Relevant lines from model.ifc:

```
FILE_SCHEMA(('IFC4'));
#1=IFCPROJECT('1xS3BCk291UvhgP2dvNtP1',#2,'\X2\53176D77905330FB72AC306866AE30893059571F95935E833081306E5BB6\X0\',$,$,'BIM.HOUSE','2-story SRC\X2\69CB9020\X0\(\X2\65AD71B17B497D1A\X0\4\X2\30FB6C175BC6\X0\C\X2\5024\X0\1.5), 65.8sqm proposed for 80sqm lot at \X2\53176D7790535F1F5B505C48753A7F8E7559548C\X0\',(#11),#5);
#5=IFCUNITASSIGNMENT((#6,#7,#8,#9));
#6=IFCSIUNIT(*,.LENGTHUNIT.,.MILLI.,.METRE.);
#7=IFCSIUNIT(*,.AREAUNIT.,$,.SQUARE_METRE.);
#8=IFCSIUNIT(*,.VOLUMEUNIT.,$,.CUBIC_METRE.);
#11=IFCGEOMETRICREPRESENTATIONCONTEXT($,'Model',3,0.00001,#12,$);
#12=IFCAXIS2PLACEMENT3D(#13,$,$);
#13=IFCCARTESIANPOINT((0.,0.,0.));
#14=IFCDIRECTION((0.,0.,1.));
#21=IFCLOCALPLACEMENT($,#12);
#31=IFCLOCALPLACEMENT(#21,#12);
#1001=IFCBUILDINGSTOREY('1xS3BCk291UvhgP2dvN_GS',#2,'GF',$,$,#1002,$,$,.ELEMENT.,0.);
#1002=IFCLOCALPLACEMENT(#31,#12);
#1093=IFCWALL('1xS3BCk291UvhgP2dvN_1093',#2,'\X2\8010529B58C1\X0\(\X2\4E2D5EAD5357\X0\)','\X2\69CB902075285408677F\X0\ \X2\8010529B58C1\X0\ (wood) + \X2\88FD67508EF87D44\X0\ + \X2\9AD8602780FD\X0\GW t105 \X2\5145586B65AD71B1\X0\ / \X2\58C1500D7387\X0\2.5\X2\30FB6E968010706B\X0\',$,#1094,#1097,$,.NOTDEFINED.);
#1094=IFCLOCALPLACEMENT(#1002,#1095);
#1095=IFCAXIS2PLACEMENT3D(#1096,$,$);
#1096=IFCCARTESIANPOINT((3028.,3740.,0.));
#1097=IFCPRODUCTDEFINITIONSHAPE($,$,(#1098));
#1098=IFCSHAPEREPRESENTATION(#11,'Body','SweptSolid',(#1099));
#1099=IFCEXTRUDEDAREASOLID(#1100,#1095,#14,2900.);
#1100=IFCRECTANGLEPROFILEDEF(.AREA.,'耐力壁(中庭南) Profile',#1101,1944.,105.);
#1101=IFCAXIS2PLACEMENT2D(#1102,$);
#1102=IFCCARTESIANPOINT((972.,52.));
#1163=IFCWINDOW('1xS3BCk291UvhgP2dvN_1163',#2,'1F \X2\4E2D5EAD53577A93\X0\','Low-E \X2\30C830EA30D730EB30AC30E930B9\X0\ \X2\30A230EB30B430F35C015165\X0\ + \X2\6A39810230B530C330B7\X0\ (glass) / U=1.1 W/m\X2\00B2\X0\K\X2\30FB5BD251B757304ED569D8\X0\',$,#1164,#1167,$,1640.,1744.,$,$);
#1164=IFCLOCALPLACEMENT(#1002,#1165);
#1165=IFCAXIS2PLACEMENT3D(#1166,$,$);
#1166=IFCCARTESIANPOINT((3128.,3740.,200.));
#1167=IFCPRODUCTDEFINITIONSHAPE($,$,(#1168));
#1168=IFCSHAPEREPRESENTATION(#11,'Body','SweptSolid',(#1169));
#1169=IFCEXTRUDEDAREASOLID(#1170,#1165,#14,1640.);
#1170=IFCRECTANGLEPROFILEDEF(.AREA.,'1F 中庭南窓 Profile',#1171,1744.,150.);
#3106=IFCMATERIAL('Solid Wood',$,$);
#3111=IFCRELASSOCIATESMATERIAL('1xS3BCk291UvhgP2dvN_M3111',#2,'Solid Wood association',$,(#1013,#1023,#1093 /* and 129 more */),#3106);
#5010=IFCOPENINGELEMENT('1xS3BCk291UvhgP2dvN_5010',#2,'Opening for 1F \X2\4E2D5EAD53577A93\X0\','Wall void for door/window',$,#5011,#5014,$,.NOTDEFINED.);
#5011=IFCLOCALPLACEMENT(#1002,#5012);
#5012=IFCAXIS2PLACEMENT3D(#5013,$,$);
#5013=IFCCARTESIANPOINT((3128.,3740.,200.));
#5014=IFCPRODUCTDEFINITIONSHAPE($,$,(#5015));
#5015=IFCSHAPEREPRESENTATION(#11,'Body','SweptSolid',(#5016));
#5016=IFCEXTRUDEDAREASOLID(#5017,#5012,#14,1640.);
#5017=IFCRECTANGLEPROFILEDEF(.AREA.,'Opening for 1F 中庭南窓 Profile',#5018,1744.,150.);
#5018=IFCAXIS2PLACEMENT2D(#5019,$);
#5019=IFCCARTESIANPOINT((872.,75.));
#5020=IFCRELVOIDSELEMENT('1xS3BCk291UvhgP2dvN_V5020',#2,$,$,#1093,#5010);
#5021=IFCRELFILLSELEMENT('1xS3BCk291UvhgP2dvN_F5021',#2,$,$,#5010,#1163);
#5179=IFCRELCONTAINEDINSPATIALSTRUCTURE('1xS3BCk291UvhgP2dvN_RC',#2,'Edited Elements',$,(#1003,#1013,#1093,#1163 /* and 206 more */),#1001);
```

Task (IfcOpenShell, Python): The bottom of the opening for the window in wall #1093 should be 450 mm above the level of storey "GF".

```python
import numpy as np
import ifcopenshell
import ifcopenshell.api.geometry
import ifcopenshell.geom
import ifcopenshell.util.element
import ifcopenshell.util.placement
import ifcopenshell.util.shape
import ifcopenshell.util.unit

model = ifcopenshell.open("model.ifc")
unit_scale = ifcopenshell.util.unit.calculate_unit_scale(model)

window = model.by_id(1163)
opening = window.FillsVoids[0].RelatingOpeningElement
storey = ifcopenshell.util.element.get_container(window, ifc_class="IfcBuildingStorey")
level = ifcopenshell.util.placement.get_local_placement(storey.ObjectPlacement)[2, 3]

# The opening's origin need not be at the sill, so measure its lowest point.
shape = ifcopenshell.geom.create_shape(ifcopenshell.geom.settings(), opening)
bottom = ifcopenshell.util.shape.get_shape_bottom_elevation(shape, shape.geometry) / unit_scale
dz = level + 450.0 - bottom

shift = np.array([0.0, 0.0, dz])
# The window is not placed relative to its opening, so move both.
for product in (opening, window):
    matrix = ifcopenshell.util.placement.get_local_placement(product.ObjectPlacement)
    matrix[:3, 3] += shift
    ifcopenshell.api.geometry.edit_object_placement(model, product=product, matrix=matrix, is_si=False)

print(f"moved by {dz * unit_scale:+.3f} m")

model.write("model_updated.ifc")
```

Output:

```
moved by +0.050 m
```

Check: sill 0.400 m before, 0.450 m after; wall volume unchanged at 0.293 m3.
